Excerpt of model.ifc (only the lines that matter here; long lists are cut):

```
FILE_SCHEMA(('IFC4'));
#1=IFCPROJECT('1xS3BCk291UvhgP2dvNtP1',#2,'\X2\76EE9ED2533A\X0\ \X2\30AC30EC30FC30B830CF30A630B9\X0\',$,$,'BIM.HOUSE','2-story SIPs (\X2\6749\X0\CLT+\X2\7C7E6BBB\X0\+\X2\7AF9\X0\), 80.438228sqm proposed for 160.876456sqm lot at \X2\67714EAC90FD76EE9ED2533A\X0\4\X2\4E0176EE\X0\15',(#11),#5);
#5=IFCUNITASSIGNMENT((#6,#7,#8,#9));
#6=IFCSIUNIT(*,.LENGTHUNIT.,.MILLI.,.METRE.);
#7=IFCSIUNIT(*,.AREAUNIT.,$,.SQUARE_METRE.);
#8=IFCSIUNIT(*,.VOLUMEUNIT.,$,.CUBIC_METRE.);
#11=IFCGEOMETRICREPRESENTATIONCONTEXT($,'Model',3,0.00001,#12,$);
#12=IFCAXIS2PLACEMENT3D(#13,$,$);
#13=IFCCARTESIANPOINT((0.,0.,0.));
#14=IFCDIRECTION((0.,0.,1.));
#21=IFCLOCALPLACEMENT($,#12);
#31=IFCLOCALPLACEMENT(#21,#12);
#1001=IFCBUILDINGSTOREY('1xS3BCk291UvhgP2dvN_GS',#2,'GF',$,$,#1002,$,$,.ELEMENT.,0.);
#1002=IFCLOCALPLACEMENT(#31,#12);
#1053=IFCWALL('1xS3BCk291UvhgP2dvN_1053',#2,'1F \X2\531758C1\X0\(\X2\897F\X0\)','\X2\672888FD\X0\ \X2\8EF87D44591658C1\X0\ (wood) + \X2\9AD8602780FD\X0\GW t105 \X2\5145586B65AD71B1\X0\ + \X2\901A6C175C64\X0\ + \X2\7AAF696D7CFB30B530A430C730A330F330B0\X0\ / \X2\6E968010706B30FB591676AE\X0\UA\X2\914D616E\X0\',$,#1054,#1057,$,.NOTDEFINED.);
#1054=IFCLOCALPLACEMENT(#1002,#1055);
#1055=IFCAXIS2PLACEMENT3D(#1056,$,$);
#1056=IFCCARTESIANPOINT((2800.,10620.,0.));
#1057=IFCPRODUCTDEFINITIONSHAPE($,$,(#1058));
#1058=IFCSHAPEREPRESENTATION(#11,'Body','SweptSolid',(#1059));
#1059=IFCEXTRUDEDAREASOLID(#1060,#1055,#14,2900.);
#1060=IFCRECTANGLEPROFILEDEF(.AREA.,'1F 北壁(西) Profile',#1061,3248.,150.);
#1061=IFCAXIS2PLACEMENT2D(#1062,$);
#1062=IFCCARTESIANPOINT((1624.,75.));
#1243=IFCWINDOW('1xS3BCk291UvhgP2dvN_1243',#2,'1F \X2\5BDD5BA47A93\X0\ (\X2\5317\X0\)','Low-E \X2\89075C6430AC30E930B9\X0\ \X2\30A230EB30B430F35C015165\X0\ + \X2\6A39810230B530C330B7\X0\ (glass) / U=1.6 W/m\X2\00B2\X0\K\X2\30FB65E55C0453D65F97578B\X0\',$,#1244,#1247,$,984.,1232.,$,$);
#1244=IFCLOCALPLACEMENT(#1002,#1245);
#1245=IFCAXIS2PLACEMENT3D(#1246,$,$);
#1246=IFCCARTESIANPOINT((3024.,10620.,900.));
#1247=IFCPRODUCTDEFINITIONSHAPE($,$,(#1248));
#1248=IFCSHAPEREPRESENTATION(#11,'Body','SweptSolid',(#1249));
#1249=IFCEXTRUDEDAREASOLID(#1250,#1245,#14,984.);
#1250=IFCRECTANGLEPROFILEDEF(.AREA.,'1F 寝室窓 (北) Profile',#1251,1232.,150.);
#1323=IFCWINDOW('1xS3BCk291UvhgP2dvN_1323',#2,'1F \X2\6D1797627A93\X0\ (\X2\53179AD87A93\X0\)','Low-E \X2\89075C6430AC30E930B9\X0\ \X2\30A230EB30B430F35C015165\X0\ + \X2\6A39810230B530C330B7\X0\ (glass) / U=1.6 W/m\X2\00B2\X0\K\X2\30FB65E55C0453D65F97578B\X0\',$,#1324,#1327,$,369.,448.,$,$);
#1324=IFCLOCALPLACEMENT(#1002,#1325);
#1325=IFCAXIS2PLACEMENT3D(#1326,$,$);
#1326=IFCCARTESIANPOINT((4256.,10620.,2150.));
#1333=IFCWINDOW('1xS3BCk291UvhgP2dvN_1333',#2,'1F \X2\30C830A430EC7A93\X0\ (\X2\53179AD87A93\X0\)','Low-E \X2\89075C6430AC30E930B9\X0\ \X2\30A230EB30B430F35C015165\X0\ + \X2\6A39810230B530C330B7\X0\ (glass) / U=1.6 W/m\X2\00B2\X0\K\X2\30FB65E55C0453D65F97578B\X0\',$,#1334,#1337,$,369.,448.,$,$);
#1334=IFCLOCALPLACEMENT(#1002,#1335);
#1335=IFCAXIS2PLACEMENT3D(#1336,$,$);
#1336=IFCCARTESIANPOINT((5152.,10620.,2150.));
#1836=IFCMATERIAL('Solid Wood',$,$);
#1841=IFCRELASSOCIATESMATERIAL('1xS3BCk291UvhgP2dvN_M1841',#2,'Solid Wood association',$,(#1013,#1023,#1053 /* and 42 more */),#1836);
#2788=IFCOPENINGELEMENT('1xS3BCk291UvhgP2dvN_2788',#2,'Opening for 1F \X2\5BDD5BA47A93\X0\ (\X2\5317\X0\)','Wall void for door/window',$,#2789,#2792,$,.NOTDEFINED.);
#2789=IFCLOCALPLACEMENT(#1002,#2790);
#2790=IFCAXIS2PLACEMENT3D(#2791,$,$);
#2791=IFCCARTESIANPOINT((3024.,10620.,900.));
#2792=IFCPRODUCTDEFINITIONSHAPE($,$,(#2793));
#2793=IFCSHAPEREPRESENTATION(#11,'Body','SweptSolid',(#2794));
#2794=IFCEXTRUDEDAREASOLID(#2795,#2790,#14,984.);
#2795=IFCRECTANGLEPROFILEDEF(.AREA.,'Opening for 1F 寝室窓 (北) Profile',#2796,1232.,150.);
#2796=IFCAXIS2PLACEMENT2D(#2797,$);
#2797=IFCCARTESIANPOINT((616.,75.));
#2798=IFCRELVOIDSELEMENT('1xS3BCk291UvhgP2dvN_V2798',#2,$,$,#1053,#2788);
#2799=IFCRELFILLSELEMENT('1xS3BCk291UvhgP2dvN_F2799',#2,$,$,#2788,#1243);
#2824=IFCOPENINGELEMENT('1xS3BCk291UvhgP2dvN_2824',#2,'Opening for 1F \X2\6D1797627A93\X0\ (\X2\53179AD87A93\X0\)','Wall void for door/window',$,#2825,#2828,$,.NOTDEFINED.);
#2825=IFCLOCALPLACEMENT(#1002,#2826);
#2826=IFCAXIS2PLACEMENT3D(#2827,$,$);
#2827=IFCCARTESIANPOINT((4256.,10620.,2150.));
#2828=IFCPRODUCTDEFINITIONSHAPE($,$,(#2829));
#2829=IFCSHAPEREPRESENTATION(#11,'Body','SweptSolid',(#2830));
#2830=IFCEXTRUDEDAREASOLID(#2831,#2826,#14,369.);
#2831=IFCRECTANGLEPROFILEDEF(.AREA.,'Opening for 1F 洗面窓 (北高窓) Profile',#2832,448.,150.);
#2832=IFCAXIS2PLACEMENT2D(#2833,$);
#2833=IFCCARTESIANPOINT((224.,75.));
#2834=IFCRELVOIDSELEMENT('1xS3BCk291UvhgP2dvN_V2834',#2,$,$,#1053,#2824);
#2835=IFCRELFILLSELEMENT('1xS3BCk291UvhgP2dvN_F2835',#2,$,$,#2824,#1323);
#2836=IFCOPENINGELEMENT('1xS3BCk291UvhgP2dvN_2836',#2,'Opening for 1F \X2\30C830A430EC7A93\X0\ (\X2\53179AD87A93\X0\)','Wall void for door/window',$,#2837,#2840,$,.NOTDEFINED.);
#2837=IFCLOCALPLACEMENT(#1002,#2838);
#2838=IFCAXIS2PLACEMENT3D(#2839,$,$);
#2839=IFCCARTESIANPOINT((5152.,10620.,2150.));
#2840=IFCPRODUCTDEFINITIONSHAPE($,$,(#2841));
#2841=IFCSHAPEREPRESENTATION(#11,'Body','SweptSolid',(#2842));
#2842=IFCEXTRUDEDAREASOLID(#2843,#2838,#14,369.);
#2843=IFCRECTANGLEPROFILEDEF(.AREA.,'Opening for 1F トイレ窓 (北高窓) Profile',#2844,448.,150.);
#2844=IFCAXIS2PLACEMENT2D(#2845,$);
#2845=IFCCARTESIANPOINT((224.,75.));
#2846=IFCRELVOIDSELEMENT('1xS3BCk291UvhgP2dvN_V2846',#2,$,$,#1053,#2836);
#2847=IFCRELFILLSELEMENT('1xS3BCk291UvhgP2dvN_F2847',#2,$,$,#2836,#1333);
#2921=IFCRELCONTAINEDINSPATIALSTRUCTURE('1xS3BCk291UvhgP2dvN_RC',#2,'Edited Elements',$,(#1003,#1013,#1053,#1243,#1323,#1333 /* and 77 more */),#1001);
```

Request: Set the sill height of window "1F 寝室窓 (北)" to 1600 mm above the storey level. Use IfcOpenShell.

```python
import numpy as np
import ifcopenshell
import ifcopenshell.api.geometry
import ifcopenshell.geom
import ifcopenshell.util.element
import ifcopenshell.util.placement
import ifcopenshell.util.shape
import ifcopenshell.util.unit

model = ifcopenshell.open("model.ifc")
unit_scale = ifcopenshell.util.unit.calculate_unit_scale(model)

window = model.by_guid("1xS3BCk291UvhgP2dvN_1243")
opening = window.FillsVoids[0].RelatingOpeningElement
storey = ifcopenshell.util.element.get_container(window, ifc_class="IfcBuildingStorey")
level = ifcopenshell.util.placement.get_local_placement(storey.ObjectPlacement)[2, 3]

# The opening's origin need not be at the sill, so measure its lowest point.
shape = ifcopenshell.geom.create_shape(ifcopenshell.geom.settings(), opening)
bottom = ifcopenshell.util.shape.get_shape_bottom_elevation(shape, shape.geometry) / unit_scale
dz = level + 1.6 / unit_scale - bottom

shift = np.array([0.0, 0.0, dz])
# The window is not placed relative to its opening, so move both.
for product in (opening, window):
    matrix = ifcopenshell.util.placement.get_local_placement(product.ObjectPlacement)
    matrix[:3, 3] += shift
    ifcopenshell.api.geometry.edit_object_placement(model, product=product, matrix=matrix, is_si=False)

print(f"moved by {dz * unit_scale:+.3f} m")

model.write("model-out.ifc")
```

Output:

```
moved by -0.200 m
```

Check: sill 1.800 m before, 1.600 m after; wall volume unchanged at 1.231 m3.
